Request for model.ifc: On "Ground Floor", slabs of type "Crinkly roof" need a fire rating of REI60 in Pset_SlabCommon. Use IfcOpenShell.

First a look at what the model holds.

```python
import ifcopenshell
import ifcopenshell.util.element

model = ifcopenshell.open("model.ifc")
print(model.schema)
storey = next(s for s in model.by_type("IfcBuildingStorey") if s.Name == "Ground Floor")
slabs = [e for e in ifcopenshell.util.element.get_decomposition(storey) if e.is_a("IfcSlab")]
seen = {}
for e in slabs:
    element_type = ifcopenshell.util.element.get_type(e)
    key = (element_type.Name if element_type != e and element_type else None, ifcopenshell.util.element.get_pset(e, "Pset_SlabCommon", "FireRating"))
    seen[key] = seen.get(key, 0) + 1
for (name, value), count in sorted(seen.items(), key=str):
    print(count, "x", name, "|", value)
```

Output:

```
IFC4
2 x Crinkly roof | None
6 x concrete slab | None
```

```python
import ifcopenshell
import ifcopenshell.api.pset
import ifcopenshell.util.element

model = ifcopenshell.open("model.ifc")

storey = next(s for s in model.by_type("IfcBuildingStorey") if s.Name == "Ground Floor")
slabs = [e for e in ifcopenshell.util.element.get_decomposition(storey) if e.is_a("IfcSlab")]

count = 0
for e in slabs:
    element_type = ifcopenshell.util.element.get_type(e)
    if element_type in (None, e) or element_type.Name != "Crinkly roof":
        continue
    # add_pset returns the element's existing set when there is one.
    pset = ifcopenshell.api.pset.add_pset(model, product=e, name="Pset_SlabCommon")
    ifcopenshell.api.pset.edit_pset(model, pset=pset, properties={"FireRating": "REI60"})
    count += 1

print(count, "slabs updated")

model.write("model_rev.ifc")
```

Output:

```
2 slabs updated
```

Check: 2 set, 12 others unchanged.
